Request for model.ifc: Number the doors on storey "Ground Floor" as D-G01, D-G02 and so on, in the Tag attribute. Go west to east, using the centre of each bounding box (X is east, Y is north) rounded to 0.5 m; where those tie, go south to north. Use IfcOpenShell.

First a look at what the model holds.

```python
import ifcopenshell
import ifcopenshell.util.element
import ifcopenshell.util.placement

model = ifcopenshell.open("model.ifc")
print(model.schema)
storey = next(s for s in model.by_type("IfcBuildingStorey") if s.Name == "Ground Floor")
doors = [e for e in ifcopenshell.util.element.get_decomposition(storey) if e.is_a("IfcDoor")]
for e in sorted(doors, key=lambda e: e.id()):
    origin = ifcopenshell.util.placement.get_local_placement(e.ObjectPlacement)[:3, 3]
    print(e.id(), e.Tag, e.Name, origin.round(2) + 0.0, sep=" | ")
```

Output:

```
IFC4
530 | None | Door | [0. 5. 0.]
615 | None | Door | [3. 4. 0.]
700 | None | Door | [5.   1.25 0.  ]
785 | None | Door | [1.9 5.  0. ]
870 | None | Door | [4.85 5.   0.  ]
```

```python
import ifcopenshell
import ifcopenshell.geom
import ifcopenshell.util.element
import ifcopenshell.util.shape

model = ifcopenshell.open("model.ifc")
settings = ifcopenshell.geom.settings()
settings.set("use-world-coords", True)


def centre(element):
    shape = ifcopenshell.geom.create_shape(settings, element)
    return ifcopenshell.util.shape.get_bbox_centroid(shape.geometry)


storey = next(s for s in model.by_type("IfcBuildingStorey") if s.Name == "Ground Floor")
doors = [e for e in ifcopenshell.util.element.get_decomposition(storey) if e.is_a("IfcDoor")]

# Insertion points can sit at a corner or the storey origin, so sort by the geometry (in metres).
centres = {e: centre(e) for e in doors}
doors.sort(key=lambda e: (round(centres[e][0] / 0.5), centres[e][1]))

for i, e in enumerate(doors, start=1):
    number = f"D-G{i:02d}"
    e.Tag = number
    print(e.id(), number)

model.write("model_v2.ifc")
```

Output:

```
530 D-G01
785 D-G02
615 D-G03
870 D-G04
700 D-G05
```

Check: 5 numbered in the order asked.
